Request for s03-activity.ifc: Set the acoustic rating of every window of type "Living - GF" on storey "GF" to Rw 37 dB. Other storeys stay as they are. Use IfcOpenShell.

First a look at what the model holds.

```python
import ifcopenshell
import ifcopenshell.util.element

model = ifcopenshell.open("s03-activity.ifc")
print(model.schema)
storey = next(s for s in model.by_type("IfcBuildingStorey") if s.Name == "GF")
windows = [e for e in ifcopenshell.util.element.get_decomposition(storey) if e.is_a("IfcWindow")]
seen = {}
for e in windows:
    element_type = ifcopenshell.util.element.get_type(e)
    key = (element_type.Name if element_type != e and element_type else None, ifcopenshell.util.element.get_pset(e, "Pset_WindowCommon", "AcousticRating"))
    seen[key] = seen.get(key, 0) + 1
for (name, value), count in sorted(seen.items(), key=str):
    print(count, "x", name, "|", value)
```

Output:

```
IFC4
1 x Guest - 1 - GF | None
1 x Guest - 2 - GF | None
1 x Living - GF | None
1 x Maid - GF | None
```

```python
import ifcopenshell
import ifcopenshell.api.pset
import ifcopenshell.util.element

model = ifcopenshell.open("s03-activity.ifc")

storey = next(s for s in model.by_type("IfcBuildingStorey") if s.Name == "GF")
windows = [e for e in ifcopenshell.util.element.get_decomposition(storey) if e.is_a("IfcWindow")]

count = 0
for e in windows:
    element_type = ifcopenshell.util.element.get_type(e)
    if element_type in (None, e) or element_type.Name != "Living - GF":
        continue
    # add_pset returns the element's existing set when there is one.
    pset = ifcopenshell.api.pset.add_pset(model, product=e, name="Pset_WindowCommon")
    ifcopenshell.api.pset.edit_pset(model, pset=pset, properties={"AcousticRating": "Rw 37 dB"})
    count += 1

print(count, "windows updated")

model.write("s03-activity_updated.ifc")
```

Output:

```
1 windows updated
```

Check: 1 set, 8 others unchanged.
